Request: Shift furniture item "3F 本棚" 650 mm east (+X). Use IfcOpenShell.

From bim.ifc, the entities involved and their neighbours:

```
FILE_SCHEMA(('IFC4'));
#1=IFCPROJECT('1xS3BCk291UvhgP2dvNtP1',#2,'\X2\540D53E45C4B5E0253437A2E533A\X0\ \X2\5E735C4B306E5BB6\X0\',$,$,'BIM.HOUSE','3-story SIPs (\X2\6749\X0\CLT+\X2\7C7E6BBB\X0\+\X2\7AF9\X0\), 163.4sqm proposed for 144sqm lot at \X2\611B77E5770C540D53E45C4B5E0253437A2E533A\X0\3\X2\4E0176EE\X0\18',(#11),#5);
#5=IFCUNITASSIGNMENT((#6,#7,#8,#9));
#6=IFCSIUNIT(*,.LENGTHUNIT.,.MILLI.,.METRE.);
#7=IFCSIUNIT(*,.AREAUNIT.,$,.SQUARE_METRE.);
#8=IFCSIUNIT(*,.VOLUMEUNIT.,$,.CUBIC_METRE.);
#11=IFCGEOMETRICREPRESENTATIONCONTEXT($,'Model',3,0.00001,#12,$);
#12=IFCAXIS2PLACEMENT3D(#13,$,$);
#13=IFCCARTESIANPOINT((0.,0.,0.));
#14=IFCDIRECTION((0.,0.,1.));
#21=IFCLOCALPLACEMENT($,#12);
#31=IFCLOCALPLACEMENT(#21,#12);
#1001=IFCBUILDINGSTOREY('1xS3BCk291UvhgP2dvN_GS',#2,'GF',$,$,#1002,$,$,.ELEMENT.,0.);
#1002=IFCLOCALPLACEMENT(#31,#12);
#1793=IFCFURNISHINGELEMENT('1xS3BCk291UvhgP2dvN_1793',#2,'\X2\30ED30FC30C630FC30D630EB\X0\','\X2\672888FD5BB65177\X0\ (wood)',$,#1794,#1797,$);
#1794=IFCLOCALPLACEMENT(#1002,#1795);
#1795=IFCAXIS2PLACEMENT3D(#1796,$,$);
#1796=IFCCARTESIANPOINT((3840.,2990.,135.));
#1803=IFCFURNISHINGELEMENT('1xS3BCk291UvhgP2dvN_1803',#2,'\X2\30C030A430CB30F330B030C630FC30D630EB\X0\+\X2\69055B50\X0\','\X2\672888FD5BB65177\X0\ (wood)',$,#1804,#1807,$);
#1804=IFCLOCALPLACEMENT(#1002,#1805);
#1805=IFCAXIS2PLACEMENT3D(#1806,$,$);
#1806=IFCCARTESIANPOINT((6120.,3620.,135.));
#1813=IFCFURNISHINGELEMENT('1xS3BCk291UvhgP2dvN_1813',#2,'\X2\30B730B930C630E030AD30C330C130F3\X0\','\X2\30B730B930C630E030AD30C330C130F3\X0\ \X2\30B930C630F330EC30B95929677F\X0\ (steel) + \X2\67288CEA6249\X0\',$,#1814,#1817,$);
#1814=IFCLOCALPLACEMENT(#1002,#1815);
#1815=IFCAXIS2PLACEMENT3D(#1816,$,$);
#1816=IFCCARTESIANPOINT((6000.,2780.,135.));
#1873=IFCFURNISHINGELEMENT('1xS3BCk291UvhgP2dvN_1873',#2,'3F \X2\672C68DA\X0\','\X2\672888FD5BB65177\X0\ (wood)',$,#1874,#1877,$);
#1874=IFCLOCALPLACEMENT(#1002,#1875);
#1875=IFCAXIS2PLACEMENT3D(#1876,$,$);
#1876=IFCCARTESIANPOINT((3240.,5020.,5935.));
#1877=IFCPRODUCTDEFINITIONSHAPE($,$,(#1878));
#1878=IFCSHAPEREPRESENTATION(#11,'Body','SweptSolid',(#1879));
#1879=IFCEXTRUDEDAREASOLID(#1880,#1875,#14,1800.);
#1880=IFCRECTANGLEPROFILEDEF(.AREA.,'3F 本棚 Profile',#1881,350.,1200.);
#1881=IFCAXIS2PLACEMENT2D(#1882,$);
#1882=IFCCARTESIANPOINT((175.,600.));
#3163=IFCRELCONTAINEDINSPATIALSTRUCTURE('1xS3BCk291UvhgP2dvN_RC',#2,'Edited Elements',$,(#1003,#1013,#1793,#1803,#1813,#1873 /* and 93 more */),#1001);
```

```python
import ifcopenshell
import ifcopenshell.api.geometry
import ifcopenshell.util.placement

model = ifcopenshell.open("bim.ifc")

item = model.by_id(1873)
matrix = ifcopenshell.util.placement.get_local_placement(item.ObjectPlacement)
matrix[0, 3] += 650.0
ifcopenshell.api.geometry.edit_object_placement(model, product=item, matrix=matrix, is_si=False)

print(ifcopenshell.util.placement.get_local_placement(item.ObjectPlacement).round(3) + 0.0)

model.write("bim-out.ifc")
```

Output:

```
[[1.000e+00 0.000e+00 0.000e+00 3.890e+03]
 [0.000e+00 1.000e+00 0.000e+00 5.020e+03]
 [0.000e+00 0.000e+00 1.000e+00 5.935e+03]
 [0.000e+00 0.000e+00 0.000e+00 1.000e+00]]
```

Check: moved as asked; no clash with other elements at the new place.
